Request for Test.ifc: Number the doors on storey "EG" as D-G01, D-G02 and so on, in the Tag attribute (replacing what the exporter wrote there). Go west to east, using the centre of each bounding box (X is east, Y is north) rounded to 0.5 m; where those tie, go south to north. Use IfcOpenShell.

First a look at what the model holds.

```python
import ifcopenshell
import ifcopenshell.util.element
import ifcopenshell.util.placement

model = ifcopenshell.open("Test.ifc")
print(model.schema)
storey = next(s for s in model.by_type("IfcBuildingStorey") if s.Name == "EG")
doors = [e for e in ifcopenshell.util.element.get_decomposition(storey) if e.is_a("IfcDoor")]
for e in sorted(doors, key=lambda e: e.id()):
    origin = ifcopenshell.util.placement.get_local_placement(e.ObjectPlacement)[:3, 3]
    print(e.id(), e.Tag, e.Name, origin.round(2) + 0.0, sep=" | ")
```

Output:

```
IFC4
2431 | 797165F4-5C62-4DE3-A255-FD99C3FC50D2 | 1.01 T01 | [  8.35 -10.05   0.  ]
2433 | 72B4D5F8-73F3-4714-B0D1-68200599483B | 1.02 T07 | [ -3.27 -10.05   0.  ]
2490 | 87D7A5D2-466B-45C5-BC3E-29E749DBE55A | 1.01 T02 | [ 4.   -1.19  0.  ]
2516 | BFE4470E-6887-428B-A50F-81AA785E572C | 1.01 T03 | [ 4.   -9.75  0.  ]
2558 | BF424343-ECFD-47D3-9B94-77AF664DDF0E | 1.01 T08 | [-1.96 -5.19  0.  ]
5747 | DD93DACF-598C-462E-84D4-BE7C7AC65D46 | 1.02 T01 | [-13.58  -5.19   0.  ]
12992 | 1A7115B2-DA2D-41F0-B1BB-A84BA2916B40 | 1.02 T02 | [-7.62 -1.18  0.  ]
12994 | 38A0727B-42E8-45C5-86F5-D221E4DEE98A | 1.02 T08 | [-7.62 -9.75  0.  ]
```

```python
import ifcopenshell
import ifcopenshell.geom
import ifcopenshell.util.element
import ifcopenshell.util.shape

model = ifcopenshell.open("Test.ifc")
settings = ifcopenshell.geom.settings()
settings.set("use-world-coords", True)


def centre(element):
    shape = ifcopenshell.geom.create_shape(settings, element)
    return ifcopenshell.util.shape.get_bbox_centroid(shape.geometry)


storey = next(s for s in model.by_type("IfcBuildingStorey") if s.Name == "EG")
doors = [e for e in ifcopenshell.util.element.get_decomposition(storey) if e.is_a("IfcDoor")]

# Insertion points can sit at a corner or the storey origin, so sort by the geometry (in metres).
centres = {e: centre(e) for e in doors}
doors.sort(key=lambda e: (round(centres[e][0] / 0.5), centres[e][1]))

for i, e in enumerate(doors, start=1):
    number = f"D-G{i:02d}"
    e.Tag = number
    print(e.id(), number)

model.write("Test_rev.ifc")
```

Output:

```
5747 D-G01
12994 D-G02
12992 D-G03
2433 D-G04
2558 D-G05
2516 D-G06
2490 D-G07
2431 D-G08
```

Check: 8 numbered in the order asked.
